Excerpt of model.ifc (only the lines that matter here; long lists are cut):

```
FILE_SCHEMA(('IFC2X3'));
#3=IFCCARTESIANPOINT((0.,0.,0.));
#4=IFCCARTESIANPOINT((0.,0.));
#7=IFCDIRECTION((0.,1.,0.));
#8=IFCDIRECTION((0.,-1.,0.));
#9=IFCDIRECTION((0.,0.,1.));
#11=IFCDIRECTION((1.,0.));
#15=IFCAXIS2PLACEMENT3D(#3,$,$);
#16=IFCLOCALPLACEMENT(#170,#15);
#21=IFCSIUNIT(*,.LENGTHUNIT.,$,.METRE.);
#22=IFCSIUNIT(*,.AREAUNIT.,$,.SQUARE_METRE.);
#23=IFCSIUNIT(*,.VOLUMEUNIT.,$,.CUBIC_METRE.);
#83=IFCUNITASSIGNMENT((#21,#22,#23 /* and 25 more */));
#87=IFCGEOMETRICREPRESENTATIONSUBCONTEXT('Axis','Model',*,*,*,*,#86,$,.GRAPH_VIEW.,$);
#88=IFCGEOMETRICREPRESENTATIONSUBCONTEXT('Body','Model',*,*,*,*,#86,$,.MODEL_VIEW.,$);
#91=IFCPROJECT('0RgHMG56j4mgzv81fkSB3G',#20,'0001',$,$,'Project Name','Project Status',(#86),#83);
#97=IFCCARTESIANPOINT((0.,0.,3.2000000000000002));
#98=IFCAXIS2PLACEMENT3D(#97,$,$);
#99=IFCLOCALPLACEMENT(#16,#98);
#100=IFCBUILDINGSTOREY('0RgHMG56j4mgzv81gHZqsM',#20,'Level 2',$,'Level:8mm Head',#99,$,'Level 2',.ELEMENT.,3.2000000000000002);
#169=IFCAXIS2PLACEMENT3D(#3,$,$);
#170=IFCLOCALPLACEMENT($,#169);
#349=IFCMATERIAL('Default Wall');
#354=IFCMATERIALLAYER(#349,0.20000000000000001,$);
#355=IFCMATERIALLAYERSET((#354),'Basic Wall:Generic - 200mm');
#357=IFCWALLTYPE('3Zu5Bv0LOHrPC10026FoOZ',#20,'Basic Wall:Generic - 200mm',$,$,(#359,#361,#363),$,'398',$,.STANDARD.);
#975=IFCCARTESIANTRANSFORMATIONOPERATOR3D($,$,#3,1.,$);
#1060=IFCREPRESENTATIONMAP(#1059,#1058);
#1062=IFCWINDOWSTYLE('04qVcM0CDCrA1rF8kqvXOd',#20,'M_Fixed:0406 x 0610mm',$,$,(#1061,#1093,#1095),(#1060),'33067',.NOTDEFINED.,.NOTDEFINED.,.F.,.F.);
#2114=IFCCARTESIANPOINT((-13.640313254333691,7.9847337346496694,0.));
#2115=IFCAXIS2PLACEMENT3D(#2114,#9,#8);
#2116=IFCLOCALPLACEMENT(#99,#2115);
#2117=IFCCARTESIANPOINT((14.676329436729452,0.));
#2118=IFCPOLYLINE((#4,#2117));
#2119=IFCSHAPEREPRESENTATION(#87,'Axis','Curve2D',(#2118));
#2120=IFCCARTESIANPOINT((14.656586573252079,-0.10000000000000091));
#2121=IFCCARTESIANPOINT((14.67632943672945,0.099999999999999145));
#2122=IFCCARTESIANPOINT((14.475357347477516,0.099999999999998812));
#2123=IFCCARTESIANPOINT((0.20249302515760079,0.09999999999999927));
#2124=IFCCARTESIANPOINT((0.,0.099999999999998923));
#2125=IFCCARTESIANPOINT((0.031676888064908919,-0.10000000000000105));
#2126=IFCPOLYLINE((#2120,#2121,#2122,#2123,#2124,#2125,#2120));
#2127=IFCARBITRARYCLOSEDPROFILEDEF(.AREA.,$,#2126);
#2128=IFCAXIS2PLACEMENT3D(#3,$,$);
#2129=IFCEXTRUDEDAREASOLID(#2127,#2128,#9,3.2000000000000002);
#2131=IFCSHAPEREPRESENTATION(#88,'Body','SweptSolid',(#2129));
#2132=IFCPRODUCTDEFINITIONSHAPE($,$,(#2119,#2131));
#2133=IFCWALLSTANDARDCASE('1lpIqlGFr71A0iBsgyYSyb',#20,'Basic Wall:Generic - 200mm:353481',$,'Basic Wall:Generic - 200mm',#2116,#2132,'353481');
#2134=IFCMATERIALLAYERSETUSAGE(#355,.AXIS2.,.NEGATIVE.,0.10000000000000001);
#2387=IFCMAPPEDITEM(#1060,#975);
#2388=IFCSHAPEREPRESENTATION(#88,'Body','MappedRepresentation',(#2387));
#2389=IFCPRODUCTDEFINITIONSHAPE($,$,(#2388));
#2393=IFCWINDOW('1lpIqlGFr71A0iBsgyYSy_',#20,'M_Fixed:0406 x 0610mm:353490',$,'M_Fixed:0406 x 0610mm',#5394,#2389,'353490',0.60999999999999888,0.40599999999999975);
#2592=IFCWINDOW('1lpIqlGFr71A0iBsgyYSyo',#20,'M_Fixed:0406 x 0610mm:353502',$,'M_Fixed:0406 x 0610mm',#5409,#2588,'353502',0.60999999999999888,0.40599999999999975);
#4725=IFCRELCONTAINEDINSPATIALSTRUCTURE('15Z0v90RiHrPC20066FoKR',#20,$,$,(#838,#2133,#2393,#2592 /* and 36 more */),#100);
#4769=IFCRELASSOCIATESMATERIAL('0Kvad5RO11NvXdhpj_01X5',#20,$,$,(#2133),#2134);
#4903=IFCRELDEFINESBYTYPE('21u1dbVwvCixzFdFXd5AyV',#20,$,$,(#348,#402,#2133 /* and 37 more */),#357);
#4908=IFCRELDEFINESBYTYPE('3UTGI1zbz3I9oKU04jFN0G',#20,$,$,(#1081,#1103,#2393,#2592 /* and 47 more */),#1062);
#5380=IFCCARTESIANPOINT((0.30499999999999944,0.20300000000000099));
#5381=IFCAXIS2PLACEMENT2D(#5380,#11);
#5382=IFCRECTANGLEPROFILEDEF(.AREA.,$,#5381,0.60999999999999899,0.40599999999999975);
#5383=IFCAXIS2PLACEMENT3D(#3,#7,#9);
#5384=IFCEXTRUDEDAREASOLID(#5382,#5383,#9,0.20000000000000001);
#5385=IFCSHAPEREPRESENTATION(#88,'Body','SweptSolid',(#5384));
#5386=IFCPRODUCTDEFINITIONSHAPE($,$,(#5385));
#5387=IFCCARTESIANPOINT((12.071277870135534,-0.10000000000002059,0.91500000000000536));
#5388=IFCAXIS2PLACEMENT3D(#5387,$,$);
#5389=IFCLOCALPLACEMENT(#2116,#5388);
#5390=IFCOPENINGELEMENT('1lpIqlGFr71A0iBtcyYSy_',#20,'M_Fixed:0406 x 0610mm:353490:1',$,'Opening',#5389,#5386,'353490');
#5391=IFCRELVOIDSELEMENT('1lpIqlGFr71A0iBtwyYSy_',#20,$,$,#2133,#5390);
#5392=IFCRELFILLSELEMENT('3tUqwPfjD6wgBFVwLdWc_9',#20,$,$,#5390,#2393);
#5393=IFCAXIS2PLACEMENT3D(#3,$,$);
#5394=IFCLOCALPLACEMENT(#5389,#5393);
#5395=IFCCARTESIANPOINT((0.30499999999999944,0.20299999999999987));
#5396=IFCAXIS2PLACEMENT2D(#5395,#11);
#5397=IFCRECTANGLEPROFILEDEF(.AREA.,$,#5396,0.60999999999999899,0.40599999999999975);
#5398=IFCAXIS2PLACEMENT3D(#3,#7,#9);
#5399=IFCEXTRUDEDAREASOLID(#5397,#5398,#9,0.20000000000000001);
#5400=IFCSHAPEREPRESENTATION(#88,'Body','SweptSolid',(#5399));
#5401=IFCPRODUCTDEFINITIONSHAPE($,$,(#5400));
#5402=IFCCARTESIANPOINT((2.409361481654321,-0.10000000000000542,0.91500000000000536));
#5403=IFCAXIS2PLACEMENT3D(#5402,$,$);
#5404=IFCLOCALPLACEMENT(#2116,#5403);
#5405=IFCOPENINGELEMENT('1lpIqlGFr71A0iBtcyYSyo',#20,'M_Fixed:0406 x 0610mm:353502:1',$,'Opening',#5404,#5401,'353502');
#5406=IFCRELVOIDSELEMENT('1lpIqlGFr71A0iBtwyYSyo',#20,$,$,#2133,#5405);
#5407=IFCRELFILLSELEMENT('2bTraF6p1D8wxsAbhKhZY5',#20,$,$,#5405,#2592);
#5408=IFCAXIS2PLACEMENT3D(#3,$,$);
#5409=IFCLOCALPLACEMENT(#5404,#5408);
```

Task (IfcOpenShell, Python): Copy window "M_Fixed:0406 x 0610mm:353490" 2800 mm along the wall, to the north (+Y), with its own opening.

```python
import ifcopenshell
import ifcopenshell.api.feature
import ifcopenshell.api.geometry
import ifcopenshell.api.root
import ifcopenshell.geom
import ifcopenshell.util.element
import ifcopenshell.util.placement
import ifcopenshell.util.shape

model = ifcopenshell.open("model.ifc")
settings = ifcopenshell.geom.settings()


def volume(element):
    """Net volume in cubic metres, openings subtracted."""
    shape = ifcopenshell.geom.create_shape(settings, element)
    return ifcopenshell.util.shape.get_volume(shape.geometry)


def reuse_history(source, copy):
    """copy_class also copies each property set's owner history, people and application; keep the originals."""
    for rel in copy.IsDefinedBy:
        if rel.is_a("IfcRelDefinesByProperties") and (history := rel.RelatingPropertyDefinition.OwnerHistory):
            rel.RelatingPropertyDefinition.OwnerHistory = source.OwnerHistory
            ifcopenshell.util.element.remove_deep2(model, history)


window = model.by_guid("1lpIqlGFr71A0iBsgyYSy_")
opening = window.FillsVoids[0].RelatingOpeningElement
wall = opening.VoidsElements[0].RelatingBuildingElement
before = volume(wall)
shift = ifcopenshell.util.placement.get_local_placement(wall.ObjectPlacement)[:3, 0] * -2.8

# copy_class copies the void relationship, type, container and properties, but no geometry.
new_opening = ifcopenshell.api.root.copy_class(model, product=opening)
new_opening.Representation = ifcopenshell.util.element.copy_deep(
    model, opening.Representation, exclude=["IfcGeometricRepresentationContext", "IfcRepresentationMap"]
)
new_opening.Name = "M_Fixed:0406 x 0610mm"
new_opening.Tag = None
new_window = ifcopenshell.api.root.copy_class(model, product=window)
new_window.Representation = ifcopenshell.util.element.copy_deep(
    model, window.Representation, exclude=["IfcGeometricRepresentationContext", "IfcRepresentationMap"]
)
new_window.Name = "M_Fixed:0406 x 0610mm"
new_window.Tag = None
reuse_history(window, new_window)
fills = ifcopenshell.api.feature.add_filling(model, opening=new_opening, element=new_window)
fills.OwnerHistory = new_window.OwnerHistory  # required in IFC2X3

for old, new in ((opening, new_opening), (window, new_window)):
    matrix = ifcopenshell.util.placement.get_local_placement(old.ObjectPlacement)
    matrix[:3, 3] += shift
    ifcopenshell.api.geometry.edit_object_placement(model, product=new, matrix=matrix, is_si=False)

after = volume(wall)

print(f"wall volume {before:.3f} -> {after:.3f} m3")

model.write("model-out.ifc")
```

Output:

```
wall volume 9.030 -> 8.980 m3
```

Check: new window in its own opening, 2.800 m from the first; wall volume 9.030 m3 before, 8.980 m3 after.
